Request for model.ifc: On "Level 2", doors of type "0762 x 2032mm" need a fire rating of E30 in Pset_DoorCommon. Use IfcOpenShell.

First a look at what the model holds.

```python
import ifcopenshell
import ifcopenshell.util.element

model = ifcopenshell.open("model.ifc")
print(model.schema)
storey = next(s for s in model.by_type("IfcBuildingStorey") if s.Name == "Level 2")
doors = [e for e in ifcopenshell.util.element.get_decomposition(storey) if e.is_a("IfcDoor")]
seen = {}
for e in doors:
    element_type = ifcopenshell.util.element.get_type(e)
    key = (element_type.Name if element_type != e and element_type else None, ifcopenshell.util.element.get_pset(e, "Pset_DoorCommon", "FireRating"))
    seen[key] = seen.get(key, 0) + 1
for (name, value), count in sorted(seen.items(), key=str):
    print(count, "x", name, "|", value)
```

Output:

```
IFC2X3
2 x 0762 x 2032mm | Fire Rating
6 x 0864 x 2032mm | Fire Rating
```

```python
import ifcopenshell
import ifcopenshell.api.pset
import ifcopenshell.util.element

model = ifcopenshell.open("model.ifc")

storey = next(s for s in model.by_type("IfcBuildingStorey") if s.Name == "Level 2")
doors = [e for e in ifcopenshell.util.element.get_decomposition(storey) if e.is_a("IfcDoor")]

count = 0
for e in doors:
    element_type = ifcopenshell.util.element.get_type(e)
    if element_type in (None, e) or element_type.Name != "0762 x 2032mm":
        continue
    # add_pset returns the element's existing set when there is one.
    pset = ifcopenshell.api.pset.add_pset(model, product=e, name="Pset_DoorCommon")
    ifcopenshell.api.pset.edit_pset(model, pset=pset, properties={"FireRating": "E30"})
    count += 1

print(count, "doors updated")

model.write("model-out.ifc")
```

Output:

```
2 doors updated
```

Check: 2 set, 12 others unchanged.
